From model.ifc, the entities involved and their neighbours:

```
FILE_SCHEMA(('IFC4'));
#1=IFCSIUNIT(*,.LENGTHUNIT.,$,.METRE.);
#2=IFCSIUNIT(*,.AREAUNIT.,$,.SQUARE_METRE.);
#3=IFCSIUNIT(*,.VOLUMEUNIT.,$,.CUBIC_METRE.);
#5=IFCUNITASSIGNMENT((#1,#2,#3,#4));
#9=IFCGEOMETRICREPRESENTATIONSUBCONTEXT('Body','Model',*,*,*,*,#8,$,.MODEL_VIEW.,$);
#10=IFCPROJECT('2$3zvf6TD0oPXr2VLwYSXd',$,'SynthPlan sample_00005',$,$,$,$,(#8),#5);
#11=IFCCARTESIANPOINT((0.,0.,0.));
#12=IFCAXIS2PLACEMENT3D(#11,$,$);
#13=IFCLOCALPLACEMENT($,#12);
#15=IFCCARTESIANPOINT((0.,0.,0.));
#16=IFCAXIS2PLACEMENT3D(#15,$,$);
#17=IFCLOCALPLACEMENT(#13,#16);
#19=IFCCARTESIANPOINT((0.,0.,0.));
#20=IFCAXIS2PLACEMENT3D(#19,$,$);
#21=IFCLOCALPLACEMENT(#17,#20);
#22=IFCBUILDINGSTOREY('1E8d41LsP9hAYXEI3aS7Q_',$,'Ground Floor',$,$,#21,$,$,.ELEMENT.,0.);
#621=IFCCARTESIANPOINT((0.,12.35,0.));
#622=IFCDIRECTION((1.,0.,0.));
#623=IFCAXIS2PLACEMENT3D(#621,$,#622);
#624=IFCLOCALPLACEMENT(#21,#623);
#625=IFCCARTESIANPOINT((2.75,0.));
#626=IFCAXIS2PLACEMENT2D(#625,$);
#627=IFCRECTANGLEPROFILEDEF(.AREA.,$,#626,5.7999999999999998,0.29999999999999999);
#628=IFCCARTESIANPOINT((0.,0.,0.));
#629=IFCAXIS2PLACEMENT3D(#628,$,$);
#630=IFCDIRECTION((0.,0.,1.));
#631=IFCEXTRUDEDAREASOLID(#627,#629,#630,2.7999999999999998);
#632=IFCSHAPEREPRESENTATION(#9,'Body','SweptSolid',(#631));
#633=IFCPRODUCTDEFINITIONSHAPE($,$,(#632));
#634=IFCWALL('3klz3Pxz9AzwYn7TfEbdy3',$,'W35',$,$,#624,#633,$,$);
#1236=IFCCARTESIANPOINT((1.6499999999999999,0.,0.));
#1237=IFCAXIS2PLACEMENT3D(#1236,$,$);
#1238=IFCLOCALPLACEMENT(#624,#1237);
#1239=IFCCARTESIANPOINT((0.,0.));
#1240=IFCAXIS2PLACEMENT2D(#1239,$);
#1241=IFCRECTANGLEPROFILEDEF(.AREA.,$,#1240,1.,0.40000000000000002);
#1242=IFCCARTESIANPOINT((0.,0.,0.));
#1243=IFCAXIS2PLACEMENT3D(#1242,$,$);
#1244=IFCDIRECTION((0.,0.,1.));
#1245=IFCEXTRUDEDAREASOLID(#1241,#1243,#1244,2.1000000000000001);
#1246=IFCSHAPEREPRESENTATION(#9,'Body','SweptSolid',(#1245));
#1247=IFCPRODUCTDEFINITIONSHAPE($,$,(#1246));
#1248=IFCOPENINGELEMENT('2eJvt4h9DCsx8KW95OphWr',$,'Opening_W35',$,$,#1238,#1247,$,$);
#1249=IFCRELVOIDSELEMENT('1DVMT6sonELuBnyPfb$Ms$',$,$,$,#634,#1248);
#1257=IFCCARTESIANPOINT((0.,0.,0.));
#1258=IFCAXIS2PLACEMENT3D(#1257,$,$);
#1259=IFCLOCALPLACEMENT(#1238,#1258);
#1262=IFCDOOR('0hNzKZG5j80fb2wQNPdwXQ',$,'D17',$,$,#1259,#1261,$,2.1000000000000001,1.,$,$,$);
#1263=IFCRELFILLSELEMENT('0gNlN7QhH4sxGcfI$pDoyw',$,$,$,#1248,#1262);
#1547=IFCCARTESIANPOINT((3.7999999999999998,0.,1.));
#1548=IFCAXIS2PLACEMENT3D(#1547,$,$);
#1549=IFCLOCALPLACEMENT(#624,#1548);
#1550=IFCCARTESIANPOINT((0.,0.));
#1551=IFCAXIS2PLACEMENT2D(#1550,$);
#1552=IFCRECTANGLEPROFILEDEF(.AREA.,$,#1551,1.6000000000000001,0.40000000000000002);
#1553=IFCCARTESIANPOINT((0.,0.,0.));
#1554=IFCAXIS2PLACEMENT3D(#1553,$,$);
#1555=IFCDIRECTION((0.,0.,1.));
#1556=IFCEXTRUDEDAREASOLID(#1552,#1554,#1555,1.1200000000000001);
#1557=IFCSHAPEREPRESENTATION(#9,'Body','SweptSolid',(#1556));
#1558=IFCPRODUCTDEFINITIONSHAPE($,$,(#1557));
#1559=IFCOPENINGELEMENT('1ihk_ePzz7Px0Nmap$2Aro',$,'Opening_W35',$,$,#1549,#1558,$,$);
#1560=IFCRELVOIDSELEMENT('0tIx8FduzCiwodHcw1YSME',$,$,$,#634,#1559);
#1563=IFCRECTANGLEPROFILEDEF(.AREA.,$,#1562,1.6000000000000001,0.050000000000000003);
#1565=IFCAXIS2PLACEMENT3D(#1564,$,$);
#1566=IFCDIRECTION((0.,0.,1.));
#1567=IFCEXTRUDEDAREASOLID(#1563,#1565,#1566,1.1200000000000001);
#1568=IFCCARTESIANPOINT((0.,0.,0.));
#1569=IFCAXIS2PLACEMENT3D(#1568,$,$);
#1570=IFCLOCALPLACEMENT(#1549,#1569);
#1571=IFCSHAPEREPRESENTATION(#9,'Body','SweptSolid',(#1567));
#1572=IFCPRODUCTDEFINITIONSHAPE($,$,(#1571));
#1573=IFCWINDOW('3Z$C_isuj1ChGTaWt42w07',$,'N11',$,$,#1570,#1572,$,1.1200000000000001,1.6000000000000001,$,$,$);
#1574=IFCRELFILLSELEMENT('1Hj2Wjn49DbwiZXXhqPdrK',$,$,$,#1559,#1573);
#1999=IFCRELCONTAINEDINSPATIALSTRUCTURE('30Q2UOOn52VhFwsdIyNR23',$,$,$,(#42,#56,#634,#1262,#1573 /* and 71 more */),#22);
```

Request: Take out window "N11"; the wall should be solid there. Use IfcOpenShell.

```python
import ifcopenshell
import ifcopenshell.api.feature
import ifcopenshell.api.root
import ifcopenshell.geom
import ifcopenshell.util.shape

model = ifcopenshell.open("model.ifc")
settings = ifcopenshell.geom.settings()


def volume(element):
    """Net volume in cubic metres, openings subtracted."""
    shape = ifcopenshell.geom.create_shape(settings, element)
    return ifcopenshell.util.shape.get_volume(shape.geometry)


window = model.by_guid("3Z$C_isuj1ChGTaWt42w07")
opening = window.FillsVoids[0].RelatingOpeningElement
wall = opening.VoidsElements[0].RelatingBuildingElement
before = volume(wall)

ifcopenshell.api.root.remove_product(model, product=window)
ifcopenshell.api.feature.remove_feature(model, feature=opening)

after = volume(wall)

print(f"wall volume {before:.3f} -> {after:.3f} m3")

model.write("model_v2.ifc")
```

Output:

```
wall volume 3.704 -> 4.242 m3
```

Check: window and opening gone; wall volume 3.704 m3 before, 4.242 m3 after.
